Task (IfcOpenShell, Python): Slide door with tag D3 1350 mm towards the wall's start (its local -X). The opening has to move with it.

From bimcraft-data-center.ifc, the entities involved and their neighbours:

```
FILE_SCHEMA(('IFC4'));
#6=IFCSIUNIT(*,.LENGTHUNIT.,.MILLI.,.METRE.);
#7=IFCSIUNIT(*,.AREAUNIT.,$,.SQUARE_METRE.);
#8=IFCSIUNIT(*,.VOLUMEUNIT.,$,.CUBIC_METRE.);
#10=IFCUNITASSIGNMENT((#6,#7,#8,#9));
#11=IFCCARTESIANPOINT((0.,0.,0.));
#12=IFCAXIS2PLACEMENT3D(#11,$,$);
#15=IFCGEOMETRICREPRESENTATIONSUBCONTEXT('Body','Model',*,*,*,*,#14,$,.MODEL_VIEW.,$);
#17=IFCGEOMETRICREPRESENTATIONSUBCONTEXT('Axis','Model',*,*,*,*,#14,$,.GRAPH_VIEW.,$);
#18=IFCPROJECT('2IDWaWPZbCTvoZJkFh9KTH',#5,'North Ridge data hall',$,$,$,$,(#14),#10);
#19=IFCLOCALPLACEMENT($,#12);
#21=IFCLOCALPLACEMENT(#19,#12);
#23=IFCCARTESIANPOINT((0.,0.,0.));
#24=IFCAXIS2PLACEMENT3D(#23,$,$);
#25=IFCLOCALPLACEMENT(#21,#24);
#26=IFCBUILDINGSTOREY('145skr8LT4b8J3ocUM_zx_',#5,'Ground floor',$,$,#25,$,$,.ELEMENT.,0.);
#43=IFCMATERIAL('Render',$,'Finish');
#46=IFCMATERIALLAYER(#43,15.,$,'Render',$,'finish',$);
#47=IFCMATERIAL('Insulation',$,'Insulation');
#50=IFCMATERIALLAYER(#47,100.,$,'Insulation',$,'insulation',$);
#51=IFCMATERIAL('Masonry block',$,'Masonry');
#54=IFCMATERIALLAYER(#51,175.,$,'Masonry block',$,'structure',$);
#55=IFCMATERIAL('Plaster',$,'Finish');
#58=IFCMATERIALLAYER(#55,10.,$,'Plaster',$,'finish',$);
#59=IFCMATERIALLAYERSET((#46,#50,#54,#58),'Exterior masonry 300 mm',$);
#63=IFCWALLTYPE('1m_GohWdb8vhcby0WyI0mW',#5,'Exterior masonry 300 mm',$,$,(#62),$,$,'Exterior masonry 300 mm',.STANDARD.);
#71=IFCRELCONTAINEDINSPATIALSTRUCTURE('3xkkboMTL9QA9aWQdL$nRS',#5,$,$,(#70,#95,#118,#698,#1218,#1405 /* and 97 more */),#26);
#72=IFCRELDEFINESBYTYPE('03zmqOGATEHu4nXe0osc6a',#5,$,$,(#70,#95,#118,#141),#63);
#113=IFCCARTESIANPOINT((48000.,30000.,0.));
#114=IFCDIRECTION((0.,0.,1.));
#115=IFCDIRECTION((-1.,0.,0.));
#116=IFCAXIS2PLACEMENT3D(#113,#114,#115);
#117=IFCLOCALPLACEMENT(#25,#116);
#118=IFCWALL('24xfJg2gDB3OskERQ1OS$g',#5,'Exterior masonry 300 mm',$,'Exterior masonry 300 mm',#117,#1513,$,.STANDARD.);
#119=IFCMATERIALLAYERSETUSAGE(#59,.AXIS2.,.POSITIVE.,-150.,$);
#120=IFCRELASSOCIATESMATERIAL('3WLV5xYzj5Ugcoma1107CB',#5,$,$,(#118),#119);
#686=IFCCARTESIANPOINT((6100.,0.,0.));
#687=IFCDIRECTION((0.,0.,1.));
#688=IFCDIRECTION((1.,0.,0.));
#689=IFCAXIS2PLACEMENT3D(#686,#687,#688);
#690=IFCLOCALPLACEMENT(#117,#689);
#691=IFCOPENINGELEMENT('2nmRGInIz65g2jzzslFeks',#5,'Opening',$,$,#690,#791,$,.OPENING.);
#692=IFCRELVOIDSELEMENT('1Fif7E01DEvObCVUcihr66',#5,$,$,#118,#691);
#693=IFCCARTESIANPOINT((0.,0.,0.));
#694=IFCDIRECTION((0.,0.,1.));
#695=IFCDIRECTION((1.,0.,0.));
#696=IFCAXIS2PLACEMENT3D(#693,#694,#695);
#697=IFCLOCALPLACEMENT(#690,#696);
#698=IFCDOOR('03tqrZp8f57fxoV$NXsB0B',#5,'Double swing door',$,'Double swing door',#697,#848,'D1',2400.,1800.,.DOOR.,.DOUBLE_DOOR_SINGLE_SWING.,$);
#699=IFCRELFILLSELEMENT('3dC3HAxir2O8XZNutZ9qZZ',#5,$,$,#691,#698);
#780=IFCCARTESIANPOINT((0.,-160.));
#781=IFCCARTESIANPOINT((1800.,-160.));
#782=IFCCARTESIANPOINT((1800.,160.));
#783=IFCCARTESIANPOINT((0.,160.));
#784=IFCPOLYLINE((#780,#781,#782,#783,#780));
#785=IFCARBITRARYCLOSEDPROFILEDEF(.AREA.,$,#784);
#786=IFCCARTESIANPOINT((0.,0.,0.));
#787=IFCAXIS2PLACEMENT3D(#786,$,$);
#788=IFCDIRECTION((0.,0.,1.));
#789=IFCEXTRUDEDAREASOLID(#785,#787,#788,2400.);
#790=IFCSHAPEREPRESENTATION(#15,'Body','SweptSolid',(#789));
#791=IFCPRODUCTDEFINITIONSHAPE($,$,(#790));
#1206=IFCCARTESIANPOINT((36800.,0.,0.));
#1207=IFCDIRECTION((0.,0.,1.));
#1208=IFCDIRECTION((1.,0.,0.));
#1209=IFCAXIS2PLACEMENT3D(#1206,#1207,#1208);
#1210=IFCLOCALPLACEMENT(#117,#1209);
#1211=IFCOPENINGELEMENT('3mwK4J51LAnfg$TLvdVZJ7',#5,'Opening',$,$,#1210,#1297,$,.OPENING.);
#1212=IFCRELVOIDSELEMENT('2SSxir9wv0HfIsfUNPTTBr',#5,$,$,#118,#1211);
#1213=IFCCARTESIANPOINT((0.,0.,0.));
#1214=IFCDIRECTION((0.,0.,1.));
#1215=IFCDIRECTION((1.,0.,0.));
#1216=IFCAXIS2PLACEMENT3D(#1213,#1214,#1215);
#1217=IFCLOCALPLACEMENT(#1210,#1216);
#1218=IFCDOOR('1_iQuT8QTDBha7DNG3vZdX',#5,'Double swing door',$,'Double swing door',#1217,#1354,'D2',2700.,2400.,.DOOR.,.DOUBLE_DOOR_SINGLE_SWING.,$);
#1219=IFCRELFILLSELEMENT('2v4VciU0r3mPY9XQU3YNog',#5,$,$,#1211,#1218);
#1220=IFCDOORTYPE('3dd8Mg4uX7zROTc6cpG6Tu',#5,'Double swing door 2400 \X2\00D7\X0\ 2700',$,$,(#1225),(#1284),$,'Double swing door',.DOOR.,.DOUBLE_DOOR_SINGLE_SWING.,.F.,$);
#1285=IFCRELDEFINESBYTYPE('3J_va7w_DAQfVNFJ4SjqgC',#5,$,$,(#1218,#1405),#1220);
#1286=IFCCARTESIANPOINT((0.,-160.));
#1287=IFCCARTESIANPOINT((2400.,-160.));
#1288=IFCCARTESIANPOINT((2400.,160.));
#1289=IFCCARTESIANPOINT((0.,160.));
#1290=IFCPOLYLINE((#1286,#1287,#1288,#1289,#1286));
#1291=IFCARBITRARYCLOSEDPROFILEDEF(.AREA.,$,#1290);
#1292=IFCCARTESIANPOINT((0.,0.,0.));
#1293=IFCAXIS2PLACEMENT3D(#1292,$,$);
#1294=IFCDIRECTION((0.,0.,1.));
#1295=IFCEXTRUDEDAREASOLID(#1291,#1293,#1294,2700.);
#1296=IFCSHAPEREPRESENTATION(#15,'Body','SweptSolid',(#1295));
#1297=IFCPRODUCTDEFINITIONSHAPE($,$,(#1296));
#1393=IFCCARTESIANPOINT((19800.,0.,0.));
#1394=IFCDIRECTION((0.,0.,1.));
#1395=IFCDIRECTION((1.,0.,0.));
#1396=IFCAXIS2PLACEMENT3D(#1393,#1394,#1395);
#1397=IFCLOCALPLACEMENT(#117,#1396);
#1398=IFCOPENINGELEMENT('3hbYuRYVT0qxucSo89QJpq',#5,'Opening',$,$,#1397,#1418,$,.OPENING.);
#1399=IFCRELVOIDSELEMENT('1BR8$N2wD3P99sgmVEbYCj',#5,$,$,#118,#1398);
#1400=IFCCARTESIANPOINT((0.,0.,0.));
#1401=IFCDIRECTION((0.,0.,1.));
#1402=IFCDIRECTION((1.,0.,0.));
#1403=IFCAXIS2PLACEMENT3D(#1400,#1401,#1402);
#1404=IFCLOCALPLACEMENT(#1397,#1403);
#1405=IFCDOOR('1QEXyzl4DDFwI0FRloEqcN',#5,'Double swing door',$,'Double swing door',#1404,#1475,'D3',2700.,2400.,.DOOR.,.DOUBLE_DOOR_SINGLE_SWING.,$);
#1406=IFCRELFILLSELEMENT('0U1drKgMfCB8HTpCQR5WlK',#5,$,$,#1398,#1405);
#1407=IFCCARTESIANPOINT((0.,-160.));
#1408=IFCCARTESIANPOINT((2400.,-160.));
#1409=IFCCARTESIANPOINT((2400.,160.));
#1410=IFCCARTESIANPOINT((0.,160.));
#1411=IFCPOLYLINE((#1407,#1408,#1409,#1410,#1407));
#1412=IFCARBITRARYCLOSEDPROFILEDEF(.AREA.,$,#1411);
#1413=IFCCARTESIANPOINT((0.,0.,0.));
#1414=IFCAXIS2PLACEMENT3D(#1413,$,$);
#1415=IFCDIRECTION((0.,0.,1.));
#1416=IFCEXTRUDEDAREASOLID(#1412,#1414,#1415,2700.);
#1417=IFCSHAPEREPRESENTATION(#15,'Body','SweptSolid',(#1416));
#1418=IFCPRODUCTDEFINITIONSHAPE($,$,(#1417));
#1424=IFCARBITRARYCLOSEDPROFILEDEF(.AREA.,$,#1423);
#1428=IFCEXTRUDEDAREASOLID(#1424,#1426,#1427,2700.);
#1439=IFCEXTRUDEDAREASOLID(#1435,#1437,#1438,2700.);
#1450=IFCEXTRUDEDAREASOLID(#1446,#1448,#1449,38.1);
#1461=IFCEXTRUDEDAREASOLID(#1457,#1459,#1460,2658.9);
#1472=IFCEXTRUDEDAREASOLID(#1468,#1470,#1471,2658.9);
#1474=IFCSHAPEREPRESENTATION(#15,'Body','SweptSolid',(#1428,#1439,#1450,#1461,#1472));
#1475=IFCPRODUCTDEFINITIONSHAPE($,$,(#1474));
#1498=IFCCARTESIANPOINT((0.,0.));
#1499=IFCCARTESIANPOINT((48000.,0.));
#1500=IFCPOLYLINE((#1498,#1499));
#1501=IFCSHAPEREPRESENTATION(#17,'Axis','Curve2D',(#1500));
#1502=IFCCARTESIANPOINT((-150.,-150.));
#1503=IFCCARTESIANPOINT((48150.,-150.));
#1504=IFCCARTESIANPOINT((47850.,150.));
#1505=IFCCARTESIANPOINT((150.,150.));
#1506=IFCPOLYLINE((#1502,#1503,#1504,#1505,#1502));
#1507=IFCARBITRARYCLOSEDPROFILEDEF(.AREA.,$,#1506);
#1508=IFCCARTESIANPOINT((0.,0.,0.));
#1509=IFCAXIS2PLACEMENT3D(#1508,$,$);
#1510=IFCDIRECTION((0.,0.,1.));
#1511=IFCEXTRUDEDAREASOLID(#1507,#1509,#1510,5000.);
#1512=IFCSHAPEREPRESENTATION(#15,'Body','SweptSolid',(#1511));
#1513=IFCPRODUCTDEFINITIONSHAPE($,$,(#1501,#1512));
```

```python
import ifcopenshell
import ifcopenshell.api.geometry
import ifcopenshell.util.placement

model = ifcopenshell.open("bimcraft-data-center.ifc")

door = model.by_id(1405)
opening = door.FillsVoids[0].RelatingOpeningElement
wall = opening.VoidsElements[0].RelatingBuildingElement

wall_matrix = ifcopenshell.util.placement.get_local_placement(wall.ObjectPlacement)
shift = wall_matrix[:3, 0] * -1350.0
before = ifcopenshell.util.placement.get_local_placement(door.ObjectPlacement)[:3, 3].copy()

# The door is placed relative to its opening, so it follows when the opening moves.
matrix = ifcopenshell.util.placement.get_local_placement(opening.ObjectPlacement)
matrix[:3, 3] += shift
ifcopenshell.api.geometry.edit_object_placement(
    model, product=opening, matrix=matrix, is_si=False, should_transform_children=True
)

after = ifcopenshell.util.placement.get_local_placement(door.ObjectPlacement)[:3, 3]
print("door moved by", (after - before).round(3) + 0.0)

model.write("bimcraft-data-center-out.ifc")
```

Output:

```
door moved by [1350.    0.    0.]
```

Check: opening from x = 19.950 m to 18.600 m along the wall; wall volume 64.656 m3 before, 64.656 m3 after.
